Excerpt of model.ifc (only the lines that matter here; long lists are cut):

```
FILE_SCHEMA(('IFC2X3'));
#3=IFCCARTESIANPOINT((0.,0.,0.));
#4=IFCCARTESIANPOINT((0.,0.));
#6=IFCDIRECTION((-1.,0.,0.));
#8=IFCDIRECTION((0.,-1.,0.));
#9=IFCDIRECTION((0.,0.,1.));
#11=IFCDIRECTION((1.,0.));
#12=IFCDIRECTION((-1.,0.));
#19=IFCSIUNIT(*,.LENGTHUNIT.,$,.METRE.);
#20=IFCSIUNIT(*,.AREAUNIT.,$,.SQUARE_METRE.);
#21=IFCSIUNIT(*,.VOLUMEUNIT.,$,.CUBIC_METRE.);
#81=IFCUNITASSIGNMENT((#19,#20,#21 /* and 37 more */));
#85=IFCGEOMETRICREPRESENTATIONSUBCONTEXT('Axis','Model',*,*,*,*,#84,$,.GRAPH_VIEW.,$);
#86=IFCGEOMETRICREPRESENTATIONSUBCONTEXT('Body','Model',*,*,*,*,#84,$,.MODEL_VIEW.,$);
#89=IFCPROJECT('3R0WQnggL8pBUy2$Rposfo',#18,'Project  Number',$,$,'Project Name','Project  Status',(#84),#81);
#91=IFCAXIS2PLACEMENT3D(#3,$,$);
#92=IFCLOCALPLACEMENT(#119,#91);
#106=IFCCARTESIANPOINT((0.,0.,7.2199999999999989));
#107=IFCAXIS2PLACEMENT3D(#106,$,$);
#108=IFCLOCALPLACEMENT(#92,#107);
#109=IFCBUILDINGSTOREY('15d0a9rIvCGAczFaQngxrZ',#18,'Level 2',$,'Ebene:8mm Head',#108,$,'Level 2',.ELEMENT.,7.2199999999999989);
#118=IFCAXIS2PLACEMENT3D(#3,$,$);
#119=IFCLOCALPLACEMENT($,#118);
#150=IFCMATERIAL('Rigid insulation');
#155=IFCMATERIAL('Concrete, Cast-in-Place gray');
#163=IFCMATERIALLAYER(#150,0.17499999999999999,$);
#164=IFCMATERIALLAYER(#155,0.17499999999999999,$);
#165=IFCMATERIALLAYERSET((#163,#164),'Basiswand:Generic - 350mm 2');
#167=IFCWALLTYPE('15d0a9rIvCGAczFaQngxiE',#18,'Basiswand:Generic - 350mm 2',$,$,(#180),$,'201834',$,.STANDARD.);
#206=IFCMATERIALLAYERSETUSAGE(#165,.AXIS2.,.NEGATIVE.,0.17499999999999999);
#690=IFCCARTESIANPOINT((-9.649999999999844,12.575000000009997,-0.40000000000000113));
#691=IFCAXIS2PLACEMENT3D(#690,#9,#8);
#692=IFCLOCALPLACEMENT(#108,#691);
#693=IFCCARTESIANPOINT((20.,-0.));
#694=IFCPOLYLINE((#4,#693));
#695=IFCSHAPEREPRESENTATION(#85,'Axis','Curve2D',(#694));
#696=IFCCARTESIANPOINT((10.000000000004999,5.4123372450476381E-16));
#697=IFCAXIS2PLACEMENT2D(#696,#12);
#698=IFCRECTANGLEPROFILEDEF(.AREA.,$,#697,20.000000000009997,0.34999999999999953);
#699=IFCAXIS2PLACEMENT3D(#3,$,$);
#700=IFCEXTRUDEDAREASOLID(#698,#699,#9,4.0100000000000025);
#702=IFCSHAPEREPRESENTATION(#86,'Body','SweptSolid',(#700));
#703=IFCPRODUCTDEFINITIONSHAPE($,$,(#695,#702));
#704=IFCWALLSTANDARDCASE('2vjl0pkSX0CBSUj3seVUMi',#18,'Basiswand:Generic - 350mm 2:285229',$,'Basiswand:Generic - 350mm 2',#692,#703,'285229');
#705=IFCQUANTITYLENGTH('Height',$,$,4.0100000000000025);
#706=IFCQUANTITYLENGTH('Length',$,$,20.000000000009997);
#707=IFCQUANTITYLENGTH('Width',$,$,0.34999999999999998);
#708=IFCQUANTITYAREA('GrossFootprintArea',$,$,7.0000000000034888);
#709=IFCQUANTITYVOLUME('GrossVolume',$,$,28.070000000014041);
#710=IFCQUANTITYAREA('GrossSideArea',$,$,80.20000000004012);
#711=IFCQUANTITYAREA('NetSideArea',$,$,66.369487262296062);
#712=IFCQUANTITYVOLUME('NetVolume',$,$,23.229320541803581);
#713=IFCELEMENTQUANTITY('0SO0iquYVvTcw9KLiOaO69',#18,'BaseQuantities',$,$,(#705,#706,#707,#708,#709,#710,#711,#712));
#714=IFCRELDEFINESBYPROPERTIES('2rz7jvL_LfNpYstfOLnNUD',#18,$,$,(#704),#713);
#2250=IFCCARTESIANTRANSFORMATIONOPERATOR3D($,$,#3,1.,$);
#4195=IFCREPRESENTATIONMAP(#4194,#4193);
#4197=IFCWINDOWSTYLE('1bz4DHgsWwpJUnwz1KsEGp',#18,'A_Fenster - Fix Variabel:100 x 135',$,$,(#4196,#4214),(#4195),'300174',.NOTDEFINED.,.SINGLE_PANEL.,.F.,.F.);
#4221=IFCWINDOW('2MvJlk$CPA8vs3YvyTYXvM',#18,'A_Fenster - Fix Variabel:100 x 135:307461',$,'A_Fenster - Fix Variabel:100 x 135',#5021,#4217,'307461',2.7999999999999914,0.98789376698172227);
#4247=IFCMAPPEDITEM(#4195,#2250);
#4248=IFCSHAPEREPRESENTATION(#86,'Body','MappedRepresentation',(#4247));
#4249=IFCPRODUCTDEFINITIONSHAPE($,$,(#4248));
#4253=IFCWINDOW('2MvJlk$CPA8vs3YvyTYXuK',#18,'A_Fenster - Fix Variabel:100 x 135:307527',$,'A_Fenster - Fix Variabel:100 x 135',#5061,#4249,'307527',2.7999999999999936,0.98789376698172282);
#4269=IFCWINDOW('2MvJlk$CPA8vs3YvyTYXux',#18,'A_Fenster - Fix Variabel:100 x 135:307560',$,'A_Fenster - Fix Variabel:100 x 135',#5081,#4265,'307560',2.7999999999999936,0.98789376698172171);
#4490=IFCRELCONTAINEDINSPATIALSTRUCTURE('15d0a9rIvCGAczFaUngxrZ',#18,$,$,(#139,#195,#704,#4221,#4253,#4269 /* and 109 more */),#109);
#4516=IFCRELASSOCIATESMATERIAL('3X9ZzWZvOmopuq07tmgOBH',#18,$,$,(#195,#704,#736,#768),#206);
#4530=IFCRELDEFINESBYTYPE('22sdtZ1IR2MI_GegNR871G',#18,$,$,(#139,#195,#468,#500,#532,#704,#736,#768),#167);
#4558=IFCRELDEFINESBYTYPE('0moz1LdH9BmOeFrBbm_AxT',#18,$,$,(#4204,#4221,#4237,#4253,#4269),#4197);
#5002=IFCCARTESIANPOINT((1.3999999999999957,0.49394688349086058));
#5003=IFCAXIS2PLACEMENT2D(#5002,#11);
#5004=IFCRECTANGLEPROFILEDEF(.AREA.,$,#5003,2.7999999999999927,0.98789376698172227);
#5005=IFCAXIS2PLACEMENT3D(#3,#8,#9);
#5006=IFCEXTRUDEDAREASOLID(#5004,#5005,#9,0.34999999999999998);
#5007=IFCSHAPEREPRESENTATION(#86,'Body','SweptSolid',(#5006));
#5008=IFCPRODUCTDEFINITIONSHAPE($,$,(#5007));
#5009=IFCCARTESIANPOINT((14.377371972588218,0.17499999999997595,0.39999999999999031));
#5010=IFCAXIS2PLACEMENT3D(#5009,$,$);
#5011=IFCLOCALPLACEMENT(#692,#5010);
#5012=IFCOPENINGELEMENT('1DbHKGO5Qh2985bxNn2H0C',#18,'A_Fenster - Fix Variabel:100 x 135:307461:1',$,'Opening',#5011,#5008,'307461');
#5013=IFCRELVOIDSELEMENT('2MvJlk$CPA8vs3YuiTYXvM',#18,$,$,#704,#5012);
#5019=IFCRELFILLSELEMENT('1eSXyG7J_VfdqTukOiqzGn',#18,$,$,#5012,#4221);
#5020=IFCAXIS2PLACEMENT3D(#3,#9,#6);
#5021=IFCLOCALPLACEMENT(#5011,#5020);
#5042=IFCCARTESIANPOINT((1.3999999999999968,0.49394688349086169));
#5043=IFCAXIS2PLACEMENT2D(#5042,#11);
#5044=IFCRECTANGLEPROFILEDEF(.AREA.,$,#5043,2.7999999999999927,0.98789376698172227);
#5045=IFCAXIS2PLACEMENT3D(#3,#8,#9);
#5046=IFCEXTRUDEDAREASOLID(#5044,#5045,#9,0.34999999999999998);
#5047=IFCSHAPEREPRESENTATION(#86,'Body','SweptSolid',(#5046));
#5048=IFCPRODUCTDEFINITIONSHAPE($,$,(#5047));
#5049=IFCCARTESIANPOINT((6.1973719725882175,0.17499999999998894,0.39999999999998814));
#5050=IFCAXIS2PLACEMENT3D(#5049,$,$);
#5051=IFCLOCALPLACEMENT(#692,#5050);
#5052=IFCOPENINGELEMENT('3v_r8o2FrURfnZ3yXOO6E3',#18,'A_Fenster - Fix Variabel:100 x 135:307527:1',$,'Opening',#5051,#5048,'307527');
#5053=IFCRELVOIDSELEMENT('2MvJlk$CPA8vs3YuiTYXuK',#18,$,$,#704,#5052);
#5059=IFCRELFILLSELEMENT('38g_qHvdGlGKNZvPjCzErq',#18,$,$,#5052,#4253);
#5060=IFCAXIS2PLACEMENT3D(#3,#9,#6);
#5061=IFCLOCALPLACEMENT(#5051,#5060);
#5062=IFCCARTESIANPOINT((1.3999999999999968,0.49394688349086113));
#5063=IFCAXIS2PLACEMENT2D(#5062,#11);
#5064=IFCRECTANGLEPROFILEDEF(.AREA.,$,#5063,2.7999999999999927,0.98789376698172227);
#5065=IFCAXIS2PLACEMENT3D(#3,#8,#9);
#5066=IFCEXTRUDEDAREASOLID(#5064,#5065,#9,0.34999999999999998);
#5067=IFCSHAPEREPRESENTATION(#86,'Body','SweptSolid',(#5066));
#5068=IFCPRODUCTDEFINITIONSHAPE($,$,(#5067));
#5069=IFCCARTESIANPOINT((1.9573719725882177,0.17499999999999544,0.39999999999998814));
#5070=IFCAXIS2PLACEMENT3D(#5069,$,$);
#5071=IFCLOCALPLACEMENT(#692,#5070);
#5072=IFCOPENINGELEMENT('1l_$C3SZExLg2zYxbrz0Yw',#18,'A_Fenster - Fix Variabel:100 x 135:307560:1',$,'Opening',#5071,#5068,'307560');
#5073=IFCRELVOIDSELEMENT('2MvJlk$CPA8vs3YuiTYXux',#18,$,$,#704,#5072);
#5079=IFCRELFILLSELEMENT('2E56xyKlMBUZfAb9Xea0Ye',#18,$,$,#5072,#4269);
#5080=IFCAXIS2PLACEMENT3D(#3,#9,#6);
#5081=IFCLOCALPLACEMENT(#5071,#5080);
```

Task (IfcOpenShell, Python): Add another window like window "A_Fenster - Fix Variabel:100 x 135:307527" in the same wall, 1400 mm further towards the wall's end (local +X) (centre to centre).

```python
import ifcopenshell
import ifcopenshell.api.feature
import ifcopenshell.api.geometry
import ifcopenshell.api.pset
import ifcopenshell.api.root
import ifcopenshell.geom
import ifcopenshell.util.element
import ifcopenshell.util.placement
import ifcopenshell.util.shape
import ifcopenshell.util.unit

model = ifcopenshell.open("model.ifc")
unit_scale = ifcopenshell.util.unit.calculate_unit_scale(model)
area_scale = ifcopenshell.util.unit.calculate_unit_scale(model, "AREAUNIT")
volume_scale = ifcopenshell.util.unit.calculate_unit_scale(model, "VOLUMEUNIT")
settings = ifcopenshell.geom.settings()


def volume(element):
    """Net volume in cubic metres, openings subtracted."""
    shape = ifcopenshell.geom.create_shape(settings, element)
    return ifcopenshell.util.shape.get_volume(shape.geometry)


def reuse_history(source, copy):
    """copy_class also copies each property set's owner history, people and application; keep the originals."""
    for rel in copy.IsDefinedBy:
        if rel.is_a("IfcRelDefinesByProperties") and (history := rel.RelatingPropertyDefinition.OwnerHistory):
            rel.RelatingPropertyDefinition.OwnerHistory = source.OwnerHistory
            ifcopenshell.util.element.remove_deep2(model, history)


window = model.by_id(4253)
opening = window.FillsVoids[0].RelatingOpeningElement
wall = opening.VoidsElements[0].RelatingBuildingElement
before = volume(wall)
shift = ifcopenshell.util.placement.get_local_placement(wall.ObjectPlacement)[:3, 0] * 1.4 / unit_scale

# copy_class copies the void relationship, type, container and properties, but no geometry.
new_opening = ifcopenshell.api.root.copy_class(model, product=opening)
new_opening.Representation = ifcopenshell.util.element.copy_deep(
    model, opening.Representation, exclude=["IfcGeometricRepresentationContext", "IfcRepresentationMap"]
)
new_opening.Name = "A_Fenster - Fix Variabel:100 x 135"
new_opening.Tag = None
reuse_history(opening, new_opening)
new_window = ifcopenshell.api.root.copy_class(model, product=window)
new_window.Representation = ifcopenshell.util.element.copy_deep(
    model, window.Representation, exclude=["IfcGeometricRepresentationContext", "IfcRepresentationMap"]
)
new_window.Name = "A_Fenster - Fix Variabel:100 x 135"
new_window.Tag = None
reuse_history(window, new_window)
fills = ifcopenshell.api.feature.add_filling(model, opening=new_opening, element=new_window)
fills.OwnerHistory = new_window.OwnerHistory  # required in IFC2X3

for old, new in ((opening, new_opening), (window, new_window)):
    matrix = ifcopenshell.util.placement.get_local_placement(old.ObjectPlacement)
    matrix[:3, 3] += shift
    ifcopenshell.api.geometry.edit_object_placement(model, product=new, matrix=matrix, is_si=False)

after = volume(wall)
thickness = 0.35  # wall thickness in metres

# Update the wall's stored quantities.
qto = model.by_id(ifcopenshell.util.element.get_pset(wall, "BaseQuantities", should_inherit=False)["id"])
ifcopenshell.api.pset.edit_qto(model, qto=qto, properties={
    "NetSideArea": after / thickness / area_scale,
    "NetVolume": after / volume_scale,
})

print(f"wall volume {before:.3f} -> {after:.3f} m3")

model.write("model-out.ifc")
```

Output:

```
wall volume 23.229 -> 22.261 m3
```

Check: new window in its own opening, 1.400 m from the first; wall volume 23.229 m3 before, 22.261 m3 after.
